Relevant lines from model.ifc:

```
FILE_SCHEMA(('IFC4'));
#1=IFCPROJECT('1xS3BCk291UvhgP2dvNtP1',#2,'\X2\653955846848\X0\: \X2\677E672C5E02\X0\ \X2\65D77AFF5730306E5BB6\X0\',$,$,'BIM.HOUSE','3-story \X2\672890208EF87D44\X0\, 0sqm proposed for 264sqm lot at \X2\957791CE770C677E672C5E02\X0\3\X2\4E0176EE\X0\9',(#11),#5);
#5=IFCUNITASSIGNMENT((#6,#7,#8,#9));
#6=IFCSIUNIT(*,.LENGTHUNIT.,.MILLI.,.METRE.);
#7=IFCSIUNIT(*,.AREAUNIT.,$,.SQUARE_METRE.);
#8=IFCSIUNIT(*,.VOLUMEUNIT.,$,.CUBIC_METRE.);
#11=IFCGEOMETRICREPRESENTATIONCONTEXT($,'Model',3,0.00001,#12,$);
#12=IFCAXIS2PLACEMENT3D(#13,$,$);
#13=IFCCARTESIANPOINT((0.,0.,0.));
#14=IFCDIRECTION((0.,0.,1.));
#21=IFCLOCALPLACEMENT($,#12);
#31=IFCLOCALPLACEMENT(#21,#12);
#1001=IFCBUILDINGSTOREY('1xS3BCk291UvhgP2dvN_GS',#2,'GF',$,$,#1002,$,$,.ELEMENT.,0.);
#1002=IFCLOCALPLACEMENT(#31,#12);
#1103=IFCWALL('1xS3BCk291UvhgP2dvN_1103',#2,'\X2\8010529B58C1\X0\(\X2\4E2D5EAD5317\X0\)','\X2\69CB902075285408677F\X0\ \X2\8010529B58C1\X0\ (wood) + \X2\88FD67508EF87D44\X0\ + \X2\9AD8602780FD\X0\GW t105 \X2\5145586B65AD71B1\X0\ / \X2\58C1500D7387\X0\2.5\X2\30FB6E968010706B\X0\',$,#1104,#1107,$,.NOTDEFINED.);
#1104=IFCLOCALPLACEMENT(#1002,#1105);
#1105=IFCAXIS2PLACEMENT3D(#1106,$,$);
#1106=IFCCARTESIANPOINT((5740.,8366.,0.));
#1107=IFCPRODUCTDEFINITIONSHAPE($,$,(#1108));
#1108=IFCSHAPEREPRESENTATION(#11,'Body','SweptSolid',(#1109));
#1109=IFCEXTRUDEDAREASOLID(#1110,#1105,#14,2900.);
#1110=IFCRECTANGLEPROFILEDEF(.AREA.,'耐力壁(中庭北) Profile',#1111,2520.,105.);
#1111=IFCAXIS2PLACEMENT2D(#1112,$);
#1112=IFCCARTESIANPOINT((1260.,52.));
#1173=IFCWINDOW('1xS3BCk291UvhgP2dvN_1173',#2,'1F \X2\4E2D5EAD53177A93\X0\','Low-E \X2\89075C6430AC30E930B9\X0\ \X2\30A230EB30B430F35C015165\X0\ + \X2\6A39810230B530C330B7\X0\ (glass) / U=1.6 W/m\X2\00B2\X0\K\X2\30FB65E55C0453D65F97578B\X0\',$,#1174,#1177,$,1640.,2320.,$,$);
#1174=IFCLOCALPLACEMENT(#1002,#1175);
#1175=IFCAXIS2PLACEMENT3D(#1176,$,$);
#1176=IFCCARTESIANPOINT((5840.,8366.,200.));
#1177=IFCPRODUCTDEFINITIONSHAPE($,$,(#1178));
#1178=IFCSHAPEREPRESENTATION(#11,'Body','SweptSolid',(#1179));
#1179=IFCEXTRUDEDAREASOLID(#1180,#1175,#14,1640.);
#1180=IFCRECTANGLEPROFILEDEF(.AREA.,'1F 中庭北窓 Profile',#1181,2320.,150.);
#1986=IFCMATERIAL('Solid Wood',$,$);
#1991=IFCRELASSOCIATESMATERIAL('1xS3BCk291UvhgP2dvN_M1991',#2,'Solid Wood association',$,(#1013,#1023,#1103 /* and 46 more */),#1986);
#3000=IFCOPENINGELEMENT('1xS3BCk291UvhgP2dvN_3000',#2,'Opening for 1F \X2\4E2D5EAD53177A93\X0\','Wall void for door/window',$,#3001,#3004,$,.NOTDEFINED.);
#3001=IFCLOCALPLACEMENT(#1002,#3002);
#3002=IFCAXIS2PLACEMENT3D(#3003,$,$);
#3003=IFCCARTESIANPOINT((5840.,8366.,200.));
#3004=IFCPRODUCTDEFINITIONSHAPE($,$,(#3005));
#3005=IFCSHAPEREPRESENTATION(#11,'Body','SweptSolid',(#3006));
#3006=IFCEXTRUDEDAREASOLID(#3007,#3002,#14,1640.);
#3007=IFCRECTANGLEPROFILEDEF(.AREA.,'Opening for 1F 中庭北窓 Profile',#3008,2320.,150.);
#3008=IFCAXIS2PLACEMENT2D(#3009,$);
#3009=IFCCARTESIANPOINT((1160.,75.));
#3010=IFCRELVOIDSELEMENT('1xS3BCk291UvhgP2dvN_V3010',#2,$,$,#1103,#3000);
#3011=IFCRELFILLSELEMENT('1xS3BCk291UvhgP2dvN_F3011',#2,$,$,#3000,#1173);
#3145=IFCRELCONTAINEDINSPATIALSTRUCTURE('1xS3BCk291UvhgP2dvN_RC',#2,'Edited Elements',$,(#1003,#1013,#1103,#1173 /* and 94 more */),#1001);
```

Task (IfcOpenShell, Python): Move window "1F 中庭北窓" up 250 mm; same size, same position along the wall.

```python
import numpy as np
import ifcopenshell
import ifcopenshell.api.geometry
import ifcopenshell.util.placement
import ifcopenshell.util.unit

model = ifcopenshell.open("model.ifc")
unit_scale = ifcopenshell.util.unit.calculate_unit_scale(model)

window = model.by_id(1173)
opening = window.FillsVoids[0].RelatingOpeningElement
dz = 0.25 / unit_scale

shift = np.array([0.0, 0.0, dz])
# The window is not placed relative to its opening, so move both.
for product in (opening, window):
    matrix = ifcopenshell.util.placement.get_local_placement(product.ObjectPlacement)
    matrix[:3, 3] += shift
    ifcopenshell.api.geometry.edit_object_placement(model, product=product, matrix=matrix, is_si=False)

print(f"moved by {dz * unit_scale:+.3f} m")

model.write("model_v2.ifc")
```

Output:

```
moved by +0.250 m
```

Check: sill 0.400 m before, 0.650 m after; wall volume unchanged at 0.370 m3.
